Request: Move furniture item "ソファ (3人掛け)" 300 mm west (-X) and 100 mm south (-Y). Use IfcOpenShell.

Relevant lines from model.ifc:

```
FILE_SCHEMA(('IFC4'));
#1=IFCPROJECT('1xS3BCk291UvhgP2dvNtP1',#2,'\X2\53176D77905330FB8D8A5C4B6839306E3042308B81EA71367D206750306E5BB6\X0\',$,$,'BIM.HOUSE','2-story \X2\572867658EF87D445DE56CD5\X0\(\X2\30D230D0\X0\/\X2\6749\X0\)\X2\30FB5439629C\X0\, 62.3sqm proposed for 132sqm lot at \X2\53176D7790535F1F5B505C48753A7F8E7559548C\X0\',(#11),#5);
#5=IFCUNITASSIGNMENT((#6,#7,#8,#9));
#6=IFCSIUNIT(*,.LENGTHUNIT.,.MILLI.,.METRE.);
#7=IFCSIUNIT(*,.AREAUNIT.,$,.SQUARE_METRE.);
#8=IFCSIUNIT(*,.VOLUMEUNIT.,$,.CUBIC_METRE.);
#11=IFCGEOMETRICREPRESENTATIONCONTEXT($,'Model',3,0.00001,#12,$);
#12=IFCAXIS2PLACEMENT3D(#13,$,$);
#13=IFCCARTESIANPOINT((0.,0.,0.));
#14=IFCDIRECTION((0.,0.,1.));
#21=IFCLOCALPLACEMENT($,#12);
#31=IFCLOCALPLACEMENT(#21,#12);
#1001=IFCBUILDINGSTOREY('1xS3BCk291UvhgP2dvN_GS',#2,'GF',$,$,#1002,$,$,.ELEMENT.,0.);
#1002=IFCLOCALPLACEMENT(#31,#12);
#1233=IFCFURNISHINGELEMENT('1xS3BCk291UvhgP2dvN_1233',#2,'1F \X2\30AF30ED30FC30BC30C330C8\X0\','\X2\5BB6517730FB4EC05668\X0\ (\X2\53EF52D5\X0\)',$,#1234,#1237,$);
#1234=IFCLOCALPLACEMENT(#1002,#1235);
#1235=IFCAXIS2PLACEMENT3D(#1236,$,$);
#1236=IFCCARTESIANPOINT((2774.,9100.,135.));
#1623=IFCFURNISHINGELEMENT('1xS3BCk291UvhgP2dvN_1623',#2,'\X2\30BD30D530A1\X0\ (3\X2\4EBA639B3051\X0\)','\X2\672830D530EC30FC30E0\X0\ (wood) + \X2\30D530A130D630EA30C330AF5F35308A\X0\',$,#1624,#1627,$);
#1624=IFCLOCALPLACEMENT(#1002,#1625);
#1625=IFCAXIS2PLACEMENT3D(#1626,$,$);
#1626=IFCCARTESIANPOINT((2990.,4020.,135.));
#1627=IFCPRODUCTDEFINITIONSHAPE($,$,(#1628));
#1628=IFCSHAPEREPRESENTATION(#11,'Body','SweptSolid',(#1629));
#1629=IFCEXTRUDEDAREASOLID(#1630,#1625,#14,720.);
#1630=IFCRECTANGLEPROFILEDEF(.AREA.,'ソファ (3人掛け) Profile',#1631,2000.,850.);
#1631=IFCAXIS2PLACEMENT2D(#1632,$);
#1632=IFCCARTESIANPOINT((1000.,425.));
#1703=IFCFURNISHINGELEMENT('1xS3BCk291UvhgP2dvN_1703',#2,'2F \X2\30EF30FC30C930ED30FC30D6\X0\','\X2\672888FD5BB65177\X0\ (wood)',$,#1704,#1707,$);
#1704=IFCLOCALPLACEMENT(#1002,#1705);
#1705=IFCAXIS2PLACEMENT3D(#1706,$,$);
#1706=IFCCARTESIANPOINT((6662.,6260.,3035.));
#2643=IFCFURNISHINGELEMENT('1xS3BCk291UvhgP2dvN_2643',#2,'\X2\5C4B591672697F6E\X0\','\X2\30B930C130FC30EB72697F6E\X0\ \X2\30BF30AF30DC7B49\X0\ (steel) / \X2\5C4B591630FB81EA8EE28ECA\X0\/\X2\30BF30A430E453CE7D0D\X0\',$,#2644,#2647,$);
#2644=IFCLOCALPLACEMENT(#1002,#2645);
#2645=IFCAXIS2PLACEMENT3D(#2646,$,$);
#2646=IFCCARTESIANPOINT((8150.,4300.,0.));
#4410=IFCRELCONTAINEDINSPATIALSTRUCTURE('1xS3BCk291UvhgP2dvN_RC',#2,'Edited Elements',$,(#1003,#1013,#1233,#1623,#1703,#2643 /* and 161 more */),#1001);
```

```python
import ifcopenshell
import ifcopenshell.api.geometry
import ifcopenshell.util.placement

model = ifcopenshell.open("model.ifc")

item = model.by_guid("1xS3BCk291UvhgP2dvN_1623")
matrix = ifcopenshell.util.placement.get_local_placement(item.ObjectPlacement)
matrix[0, 3] -= 300.0
matrix[1, 3] -= 100.0
ifcopenshell.api.geometry.edit_object_placement(model, product=item, matrix=matrix, is_si=False)

print(ifcopenshell.util.placement.get_local_placement(item.ObjectPlacement).round(3) + 0.0)

model.write("model-out.ifc")
```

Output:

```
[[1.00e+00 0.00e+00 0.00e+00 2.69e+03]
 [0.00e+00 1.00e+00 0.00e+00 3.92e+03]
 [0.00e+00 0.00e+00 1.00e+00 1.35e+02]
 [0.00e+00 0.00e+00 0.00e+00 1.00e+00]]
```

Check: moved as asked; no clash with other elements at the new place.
